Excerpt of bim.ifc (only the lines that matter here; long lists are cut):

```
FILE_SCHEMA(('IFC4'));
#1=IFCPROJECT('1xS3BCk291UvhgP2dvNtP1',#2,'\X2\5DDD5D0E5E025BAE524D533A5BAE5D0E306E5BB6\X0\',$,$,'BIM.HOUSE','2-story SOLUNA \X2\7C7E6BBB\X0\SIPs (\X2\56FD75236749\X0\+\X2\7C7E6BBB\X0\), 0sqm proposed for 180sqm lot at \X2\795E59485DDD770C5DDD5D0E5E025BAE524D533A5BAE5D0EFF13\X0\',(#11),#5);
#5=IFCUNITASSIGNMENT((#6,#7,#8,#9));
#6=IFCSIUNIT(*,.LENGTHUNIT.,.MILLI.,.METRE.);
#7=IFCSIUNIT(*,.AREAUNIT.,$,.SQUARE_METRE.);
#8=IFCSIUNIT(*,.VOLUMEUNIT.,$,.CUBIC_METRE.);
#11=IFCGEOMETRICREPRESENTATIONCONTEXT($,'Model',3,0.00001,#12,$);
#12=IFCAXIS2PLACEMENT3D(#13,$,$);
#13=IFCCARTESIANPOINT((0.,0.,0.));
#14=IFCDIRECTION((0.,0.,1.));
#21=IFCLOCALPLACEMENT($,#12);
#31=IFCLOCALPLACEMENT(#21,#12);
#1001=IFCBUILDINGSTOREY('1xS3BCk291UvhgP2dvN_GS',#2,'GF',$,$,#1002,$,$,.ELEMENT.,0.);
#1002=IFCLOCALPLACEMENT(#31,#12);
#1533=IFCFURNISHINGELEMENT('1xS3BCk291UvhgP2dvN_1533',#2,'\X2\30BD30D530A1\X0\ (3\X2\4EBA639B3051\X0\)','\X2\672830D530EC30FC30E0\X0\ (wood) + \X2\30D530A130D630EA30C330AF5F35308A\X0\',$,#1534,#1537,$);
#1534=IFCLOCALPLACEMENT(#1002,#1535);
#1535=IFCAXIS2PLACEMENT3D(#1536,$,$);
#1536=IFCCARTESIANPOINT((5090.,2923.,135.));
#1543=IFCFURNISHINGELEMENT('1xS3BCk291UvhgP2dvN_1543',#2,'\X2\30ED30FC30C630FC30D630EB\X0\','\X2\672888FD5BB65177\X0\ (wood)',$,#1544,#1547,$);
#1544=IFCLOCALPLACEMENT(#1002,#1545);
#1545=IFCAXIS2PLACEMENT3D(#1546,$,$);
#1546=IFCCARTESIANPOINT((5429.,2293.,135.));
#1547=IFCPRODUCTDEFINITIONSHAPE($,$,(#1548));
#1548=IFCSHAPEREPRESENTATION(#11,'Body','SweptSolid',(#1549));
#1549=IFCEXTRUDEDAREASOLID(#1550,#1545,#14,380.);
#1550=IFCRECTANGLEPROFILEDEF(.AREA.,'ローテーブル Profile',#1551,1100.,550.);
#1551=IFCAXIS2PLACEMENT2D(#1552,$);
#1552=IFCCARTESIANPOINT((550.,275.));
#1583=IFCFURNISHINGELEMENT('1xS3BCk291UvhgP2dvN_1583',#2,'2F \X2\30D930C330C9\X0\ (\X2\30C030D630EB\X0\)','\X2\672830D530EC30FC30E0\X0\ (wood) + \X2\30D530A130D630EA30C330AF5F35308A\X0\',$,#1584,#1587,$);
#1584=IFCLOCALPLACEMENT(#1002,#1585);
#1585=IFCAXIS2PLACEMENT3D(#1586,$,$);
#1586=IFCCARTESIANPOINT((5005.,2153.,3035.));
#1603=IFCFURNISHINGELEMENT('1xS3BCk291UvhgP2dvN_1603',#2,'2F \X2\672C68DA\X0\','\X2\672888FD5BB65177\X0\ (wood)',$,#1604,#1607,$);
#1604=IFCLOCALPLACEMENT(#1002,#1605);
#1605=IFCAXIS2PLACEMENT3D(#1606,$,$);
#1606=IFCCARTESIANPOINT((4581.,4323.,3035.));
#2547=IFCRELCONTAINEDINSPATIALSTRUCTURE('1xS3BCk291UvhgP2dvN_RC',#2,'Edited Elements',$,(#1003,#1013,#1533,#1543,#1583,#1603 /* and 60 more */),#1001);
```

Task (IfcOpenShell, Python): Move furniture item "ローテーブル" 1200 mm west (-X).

```python
import ifcopenshell
import ifcopenshell.api.geometry
import ifcopenshell.util.placement

model = ifcopenshell.open("bim.ifc")

item = model.by_id(1543)
matrix = ifcopenshell.util.placement.get_local_placement(item.ObjectPlacement)
matrix[0, 3] -= 1200.0
ifcopenshell.api.geometry.edit_object_placement(model, product=item, matrix=matrix, is_si=False)

print(ifcopenshell.util.placement.get_local_placement(item.ObjectPlacement).round(3) + 0.0)

model.write("bim_v2.ifc")
```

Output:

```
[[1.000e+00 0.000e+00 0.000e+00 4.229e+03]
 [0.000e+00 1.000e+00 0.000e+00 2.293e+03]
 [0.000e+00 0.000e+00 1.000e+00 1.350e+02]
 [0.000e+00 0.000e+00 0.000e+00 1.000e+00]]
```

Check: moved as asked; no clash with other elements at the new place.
